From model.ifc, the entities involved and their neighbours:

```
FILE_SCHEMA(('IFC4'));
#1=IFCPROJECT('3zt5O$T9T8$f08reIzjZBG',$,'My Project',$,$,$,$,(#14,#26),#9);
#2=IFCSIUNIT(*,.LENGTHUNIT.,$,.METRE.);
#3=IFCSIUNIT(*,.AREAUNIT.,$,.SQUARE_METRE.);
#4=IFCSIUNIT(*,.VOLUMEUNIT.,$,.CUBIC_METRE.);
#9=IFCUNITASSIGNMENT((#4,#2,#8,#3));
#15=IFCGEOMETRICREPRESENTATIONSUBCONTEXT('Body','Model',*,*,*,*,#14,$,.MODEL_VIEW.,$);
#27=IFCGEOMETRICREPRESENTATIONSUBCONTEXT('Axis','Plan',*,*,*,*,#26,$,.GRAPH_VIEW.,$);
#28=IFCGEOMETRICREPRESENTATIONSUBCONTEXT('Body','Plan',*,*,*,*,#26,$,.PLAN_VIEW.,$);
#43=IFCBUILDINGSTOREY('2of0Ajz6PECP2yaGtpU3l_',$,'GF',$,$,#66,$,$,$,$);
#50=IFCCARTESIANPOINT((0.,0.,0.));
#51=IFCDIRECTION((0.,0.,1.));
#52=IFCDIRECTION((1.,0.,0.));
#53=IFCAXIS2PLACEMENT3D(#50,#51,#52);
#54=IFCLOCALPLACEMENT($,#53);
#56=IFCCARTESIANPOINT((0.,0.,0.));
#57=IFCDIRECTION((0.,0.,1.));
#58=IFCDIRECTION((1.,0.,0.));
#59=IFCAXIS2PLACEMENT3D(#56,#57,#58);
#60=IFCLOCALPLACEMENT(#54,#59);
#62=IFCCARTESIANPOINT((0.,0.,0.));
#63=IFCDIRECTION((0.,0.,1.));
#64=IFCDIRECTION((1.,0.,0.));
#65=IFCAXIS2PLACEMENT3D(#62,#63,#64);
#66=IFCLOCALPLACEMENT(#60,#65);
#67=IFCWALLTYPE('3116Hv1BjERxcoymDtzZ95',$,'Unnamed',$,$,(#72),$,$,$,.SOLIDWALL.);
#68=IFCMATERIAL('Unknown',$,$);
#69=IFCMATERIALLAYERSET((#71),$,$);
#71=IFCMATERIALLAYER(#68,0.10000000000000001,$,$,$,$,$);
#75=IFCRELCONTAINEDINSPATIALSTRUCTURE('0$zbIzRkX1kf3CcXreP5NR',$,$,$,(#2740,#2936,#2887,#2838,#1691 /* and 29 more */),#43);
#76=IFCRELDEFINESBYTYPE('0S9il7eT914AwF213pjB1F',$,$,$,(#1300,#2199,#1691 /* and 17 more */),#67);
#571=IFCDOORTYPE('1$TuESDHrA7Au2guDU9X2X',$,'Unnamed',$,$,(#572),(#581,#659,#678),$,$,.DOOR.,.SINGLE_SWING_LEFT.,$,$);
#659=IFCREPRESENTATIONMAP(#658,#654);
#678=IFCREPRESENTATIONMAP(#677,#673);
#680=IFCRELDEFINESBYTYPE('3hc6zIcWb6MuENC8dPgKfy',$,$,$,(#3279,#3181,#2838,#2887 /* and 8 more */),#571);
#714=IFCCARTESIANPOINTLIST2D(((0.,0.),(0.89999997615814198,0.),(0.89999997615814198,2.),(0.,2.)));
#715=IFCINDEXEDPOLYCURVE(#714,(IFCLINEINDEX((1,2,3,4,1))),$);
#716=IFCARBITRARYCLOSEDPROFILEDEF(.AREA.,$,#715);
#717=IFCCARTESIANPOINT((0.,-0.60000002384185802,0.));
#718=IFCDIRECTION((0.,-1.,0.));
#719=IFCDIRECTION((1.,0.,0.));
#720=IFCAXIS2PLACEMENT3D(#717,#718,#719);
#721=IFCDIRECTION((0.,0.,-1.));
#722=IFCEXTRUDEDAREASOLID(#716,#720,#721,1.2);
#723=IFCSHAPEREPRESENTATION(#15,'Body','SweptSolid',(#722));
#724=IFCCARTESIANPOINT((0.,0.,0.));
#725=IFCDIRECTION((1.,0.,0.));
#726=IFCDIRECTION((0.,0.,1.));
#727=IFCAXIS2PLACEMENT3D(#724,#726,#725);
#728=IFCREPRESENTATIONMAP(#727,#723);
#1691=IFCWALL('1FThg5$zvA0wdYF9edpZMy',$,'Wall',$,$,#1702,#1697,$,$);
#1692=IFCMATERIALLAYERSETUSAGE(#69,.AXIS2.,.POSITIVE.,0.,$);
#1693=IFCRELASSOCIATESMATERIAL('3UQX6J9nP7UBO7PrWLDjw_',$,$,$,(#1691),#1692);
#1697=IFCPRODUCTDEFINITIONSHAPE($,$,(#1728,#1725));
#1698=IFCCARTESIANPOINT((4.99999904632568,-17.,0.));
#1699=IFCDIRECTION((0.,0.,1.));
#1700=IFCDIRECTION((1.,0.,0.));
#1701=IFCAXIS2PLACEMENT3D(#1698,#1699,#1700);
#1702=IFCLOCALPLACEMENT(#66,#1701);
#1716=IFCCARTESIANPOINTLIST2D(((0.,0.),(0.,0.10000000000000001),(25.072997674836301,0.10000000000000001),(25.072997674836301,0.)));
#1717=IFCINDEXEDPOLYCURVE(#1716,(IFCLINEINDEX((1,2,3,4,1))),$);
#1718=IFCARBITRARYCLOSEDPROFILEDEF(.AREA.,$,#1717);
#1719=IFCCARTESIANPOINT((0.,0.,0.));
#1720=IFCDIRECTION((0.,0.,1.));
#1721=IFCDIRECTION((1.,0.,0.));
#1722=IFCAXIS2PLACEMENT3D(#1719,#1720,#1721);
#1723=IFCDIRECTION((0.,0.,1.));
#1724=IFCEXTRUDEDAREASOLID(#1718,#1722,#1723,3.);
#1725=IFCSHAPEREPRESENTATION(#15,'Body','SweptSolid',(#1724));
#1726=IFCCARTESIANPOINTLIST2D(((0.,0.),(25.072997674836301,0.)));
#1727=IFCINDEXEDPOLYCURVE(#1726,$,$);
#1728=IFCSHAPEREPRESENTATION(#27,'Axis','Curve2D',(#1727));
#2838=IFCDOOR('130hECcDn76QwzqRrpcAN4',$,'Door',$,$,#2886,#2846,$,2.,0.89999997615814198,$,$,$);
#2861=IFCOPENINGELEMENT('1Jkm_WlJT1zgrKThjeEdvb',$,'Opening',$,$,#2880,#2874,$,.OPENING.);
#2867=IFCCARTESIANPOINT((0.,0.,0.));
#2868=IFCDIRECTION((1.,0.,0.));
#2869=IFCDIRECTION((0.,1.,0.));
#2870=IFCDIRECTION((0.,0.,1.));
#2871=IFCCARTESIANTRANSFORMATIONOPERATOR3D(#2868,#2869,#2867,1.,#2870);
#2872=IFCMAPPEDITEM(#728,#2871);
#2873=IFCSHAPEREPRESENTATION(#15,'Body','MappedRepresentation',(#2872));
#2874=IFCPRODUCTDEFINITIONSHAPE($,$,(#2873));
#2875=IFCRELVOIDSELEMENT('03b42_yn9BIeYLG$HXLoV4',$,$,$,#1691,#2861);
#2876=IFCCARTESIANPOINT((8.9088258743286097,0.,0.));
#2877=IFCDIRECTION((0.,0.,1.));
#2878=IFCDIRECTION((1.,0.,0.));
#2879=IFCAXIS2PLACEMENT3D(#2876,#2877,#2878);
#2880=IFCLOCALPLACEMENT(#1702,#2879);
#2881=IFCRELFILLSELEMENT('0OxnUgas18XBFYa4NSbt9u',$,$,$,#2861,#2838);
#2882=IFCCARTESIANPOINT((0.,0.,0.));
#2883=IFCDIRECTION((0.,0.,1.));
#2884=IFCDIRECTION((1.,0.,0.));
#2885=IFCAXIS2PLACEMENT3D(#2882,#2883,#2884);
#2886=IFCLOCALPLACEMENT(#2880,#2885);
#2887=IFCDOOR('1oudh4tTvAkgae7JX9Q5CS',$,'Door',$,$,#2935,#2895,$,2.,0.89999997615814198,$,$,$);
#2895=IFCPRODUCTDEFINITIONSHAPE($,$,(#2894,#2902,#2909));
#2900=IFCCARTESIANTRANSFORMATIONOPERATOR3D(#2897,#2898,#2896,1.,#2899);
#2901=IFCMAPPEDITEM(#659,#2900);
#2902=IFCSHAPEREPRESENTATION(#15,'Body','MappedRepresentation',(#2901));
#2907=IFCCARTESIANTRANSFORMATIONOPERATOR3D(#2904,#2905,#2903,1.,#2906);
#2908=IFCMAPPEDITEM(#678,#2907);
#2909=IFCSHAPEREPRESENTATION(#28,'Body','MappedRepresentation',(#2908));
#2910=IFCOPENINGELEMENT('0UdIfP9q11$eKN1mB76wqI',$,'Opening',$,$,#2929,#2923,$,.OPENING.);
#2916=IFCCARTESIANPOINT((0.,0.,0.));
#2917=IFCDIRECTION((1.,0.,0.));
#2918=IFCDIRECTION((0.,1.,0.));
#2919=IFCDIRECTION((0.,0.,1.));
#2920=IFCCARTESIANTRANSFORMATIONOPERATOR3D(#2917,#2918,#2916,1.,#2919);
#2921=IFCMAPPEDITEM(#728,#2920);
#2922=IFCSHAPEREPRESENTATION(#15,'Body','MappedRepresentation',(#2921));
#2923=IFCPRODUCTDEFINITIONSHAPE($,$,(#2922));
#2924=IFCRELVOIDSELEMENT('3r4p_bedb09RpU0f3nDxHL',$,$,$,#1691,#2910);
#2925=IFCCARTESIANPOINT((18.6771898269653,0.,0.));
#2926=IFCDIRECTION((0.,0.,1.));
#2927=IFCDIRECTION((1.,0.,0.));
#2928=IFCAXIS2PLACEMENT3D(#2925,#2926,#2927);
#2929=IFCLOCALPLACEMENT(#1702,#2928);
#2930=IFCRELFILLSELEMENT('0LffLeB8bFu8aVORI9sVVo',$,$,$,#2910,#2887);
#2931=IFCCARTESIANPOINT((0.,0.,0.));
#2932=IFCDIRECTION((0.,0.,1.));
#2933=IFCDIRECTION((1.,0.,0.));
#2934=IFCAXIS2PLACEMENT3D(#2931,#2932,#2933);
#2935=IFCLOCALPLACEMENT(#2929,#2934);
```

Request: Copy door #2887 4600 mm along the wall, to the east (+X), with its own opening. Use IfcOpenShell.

```python
import ifcopenshell
import ifcopenshell.api.feature
import ifcopenshell.api.geometry
import ifcopenshell.api.root
import ifcopenshell.geom
import ifcopenshell.util.element
import ifcopenshell.util.placement
import ifcopenshell.util.shape
import ifcopenshell.util.unit

model = ifcopenshell.open("model.ifc")
unit_scale = ifcopenshell.util.unit.calculate_unit_scale(model)
settings = ifcopenshell.geom.settings()


def volume(element):
    """Net volume in cubic metres, openings subtracted."""
    shape = ifcopenshell.geom.create_shape(settings, element)
    return ifcopenshell.util.shape.get_volume(shape.geometry)


door = model.by_guid("1oudh4tTvAkgae7JX9Q5CS")
opening = door.FillsVoids[0].RelatingOpeningElement
wall = opening.VoidsElements[0].RelatingBuildingElement
before = volume(wall)
shift = ifcopenshell.util.placement.get_local_placement(wall.ObjectPlacement)[:3, 0] * 4.6 / unit_scale

# copy_class copies the void relationship, type, container and properties, but no geometry.
new_opening = ifcopenshell.api.root.copy_class(model, product=opening)
new_opening.Representation = ifcopenshell.util.element.copy_deep(
    model, opening.Representation, exclude=["IfcGeometricRepresentationContext", "IfcRepresentationMap"]
)
new_door = ifcopenshell.api.root.copy_class(model, product=door)
new_door.Representation = ifcopenshell.util.element.copy_deep(
    model, door.Representation, exclude=["IfcGeometricRepresentationContext", "IfcRepresentationMap"]
)
ifcopenshell.api.feature.add_filling(model, opening=new_opening, element=new_door)

for old, new in ((opening, new_opening), (door, new_door)):
    matrix = ifcopenshell.util.placement.get_local_placement(old.ObjectPlacement)
    matrix[:3, 3] += shift
    ifcopenshell.api.geometry.edit_object_placement(model, product=new, matrix=matrix, is_si=False)

after = volume(wall)

print(f"wall volume {before:.3f} -> {after:.3f} m3")

model.write("model_rev.ifc")
```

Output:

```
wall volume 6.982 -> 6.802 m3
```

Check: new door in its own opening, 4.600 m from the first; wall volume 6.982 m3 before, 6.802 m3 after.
